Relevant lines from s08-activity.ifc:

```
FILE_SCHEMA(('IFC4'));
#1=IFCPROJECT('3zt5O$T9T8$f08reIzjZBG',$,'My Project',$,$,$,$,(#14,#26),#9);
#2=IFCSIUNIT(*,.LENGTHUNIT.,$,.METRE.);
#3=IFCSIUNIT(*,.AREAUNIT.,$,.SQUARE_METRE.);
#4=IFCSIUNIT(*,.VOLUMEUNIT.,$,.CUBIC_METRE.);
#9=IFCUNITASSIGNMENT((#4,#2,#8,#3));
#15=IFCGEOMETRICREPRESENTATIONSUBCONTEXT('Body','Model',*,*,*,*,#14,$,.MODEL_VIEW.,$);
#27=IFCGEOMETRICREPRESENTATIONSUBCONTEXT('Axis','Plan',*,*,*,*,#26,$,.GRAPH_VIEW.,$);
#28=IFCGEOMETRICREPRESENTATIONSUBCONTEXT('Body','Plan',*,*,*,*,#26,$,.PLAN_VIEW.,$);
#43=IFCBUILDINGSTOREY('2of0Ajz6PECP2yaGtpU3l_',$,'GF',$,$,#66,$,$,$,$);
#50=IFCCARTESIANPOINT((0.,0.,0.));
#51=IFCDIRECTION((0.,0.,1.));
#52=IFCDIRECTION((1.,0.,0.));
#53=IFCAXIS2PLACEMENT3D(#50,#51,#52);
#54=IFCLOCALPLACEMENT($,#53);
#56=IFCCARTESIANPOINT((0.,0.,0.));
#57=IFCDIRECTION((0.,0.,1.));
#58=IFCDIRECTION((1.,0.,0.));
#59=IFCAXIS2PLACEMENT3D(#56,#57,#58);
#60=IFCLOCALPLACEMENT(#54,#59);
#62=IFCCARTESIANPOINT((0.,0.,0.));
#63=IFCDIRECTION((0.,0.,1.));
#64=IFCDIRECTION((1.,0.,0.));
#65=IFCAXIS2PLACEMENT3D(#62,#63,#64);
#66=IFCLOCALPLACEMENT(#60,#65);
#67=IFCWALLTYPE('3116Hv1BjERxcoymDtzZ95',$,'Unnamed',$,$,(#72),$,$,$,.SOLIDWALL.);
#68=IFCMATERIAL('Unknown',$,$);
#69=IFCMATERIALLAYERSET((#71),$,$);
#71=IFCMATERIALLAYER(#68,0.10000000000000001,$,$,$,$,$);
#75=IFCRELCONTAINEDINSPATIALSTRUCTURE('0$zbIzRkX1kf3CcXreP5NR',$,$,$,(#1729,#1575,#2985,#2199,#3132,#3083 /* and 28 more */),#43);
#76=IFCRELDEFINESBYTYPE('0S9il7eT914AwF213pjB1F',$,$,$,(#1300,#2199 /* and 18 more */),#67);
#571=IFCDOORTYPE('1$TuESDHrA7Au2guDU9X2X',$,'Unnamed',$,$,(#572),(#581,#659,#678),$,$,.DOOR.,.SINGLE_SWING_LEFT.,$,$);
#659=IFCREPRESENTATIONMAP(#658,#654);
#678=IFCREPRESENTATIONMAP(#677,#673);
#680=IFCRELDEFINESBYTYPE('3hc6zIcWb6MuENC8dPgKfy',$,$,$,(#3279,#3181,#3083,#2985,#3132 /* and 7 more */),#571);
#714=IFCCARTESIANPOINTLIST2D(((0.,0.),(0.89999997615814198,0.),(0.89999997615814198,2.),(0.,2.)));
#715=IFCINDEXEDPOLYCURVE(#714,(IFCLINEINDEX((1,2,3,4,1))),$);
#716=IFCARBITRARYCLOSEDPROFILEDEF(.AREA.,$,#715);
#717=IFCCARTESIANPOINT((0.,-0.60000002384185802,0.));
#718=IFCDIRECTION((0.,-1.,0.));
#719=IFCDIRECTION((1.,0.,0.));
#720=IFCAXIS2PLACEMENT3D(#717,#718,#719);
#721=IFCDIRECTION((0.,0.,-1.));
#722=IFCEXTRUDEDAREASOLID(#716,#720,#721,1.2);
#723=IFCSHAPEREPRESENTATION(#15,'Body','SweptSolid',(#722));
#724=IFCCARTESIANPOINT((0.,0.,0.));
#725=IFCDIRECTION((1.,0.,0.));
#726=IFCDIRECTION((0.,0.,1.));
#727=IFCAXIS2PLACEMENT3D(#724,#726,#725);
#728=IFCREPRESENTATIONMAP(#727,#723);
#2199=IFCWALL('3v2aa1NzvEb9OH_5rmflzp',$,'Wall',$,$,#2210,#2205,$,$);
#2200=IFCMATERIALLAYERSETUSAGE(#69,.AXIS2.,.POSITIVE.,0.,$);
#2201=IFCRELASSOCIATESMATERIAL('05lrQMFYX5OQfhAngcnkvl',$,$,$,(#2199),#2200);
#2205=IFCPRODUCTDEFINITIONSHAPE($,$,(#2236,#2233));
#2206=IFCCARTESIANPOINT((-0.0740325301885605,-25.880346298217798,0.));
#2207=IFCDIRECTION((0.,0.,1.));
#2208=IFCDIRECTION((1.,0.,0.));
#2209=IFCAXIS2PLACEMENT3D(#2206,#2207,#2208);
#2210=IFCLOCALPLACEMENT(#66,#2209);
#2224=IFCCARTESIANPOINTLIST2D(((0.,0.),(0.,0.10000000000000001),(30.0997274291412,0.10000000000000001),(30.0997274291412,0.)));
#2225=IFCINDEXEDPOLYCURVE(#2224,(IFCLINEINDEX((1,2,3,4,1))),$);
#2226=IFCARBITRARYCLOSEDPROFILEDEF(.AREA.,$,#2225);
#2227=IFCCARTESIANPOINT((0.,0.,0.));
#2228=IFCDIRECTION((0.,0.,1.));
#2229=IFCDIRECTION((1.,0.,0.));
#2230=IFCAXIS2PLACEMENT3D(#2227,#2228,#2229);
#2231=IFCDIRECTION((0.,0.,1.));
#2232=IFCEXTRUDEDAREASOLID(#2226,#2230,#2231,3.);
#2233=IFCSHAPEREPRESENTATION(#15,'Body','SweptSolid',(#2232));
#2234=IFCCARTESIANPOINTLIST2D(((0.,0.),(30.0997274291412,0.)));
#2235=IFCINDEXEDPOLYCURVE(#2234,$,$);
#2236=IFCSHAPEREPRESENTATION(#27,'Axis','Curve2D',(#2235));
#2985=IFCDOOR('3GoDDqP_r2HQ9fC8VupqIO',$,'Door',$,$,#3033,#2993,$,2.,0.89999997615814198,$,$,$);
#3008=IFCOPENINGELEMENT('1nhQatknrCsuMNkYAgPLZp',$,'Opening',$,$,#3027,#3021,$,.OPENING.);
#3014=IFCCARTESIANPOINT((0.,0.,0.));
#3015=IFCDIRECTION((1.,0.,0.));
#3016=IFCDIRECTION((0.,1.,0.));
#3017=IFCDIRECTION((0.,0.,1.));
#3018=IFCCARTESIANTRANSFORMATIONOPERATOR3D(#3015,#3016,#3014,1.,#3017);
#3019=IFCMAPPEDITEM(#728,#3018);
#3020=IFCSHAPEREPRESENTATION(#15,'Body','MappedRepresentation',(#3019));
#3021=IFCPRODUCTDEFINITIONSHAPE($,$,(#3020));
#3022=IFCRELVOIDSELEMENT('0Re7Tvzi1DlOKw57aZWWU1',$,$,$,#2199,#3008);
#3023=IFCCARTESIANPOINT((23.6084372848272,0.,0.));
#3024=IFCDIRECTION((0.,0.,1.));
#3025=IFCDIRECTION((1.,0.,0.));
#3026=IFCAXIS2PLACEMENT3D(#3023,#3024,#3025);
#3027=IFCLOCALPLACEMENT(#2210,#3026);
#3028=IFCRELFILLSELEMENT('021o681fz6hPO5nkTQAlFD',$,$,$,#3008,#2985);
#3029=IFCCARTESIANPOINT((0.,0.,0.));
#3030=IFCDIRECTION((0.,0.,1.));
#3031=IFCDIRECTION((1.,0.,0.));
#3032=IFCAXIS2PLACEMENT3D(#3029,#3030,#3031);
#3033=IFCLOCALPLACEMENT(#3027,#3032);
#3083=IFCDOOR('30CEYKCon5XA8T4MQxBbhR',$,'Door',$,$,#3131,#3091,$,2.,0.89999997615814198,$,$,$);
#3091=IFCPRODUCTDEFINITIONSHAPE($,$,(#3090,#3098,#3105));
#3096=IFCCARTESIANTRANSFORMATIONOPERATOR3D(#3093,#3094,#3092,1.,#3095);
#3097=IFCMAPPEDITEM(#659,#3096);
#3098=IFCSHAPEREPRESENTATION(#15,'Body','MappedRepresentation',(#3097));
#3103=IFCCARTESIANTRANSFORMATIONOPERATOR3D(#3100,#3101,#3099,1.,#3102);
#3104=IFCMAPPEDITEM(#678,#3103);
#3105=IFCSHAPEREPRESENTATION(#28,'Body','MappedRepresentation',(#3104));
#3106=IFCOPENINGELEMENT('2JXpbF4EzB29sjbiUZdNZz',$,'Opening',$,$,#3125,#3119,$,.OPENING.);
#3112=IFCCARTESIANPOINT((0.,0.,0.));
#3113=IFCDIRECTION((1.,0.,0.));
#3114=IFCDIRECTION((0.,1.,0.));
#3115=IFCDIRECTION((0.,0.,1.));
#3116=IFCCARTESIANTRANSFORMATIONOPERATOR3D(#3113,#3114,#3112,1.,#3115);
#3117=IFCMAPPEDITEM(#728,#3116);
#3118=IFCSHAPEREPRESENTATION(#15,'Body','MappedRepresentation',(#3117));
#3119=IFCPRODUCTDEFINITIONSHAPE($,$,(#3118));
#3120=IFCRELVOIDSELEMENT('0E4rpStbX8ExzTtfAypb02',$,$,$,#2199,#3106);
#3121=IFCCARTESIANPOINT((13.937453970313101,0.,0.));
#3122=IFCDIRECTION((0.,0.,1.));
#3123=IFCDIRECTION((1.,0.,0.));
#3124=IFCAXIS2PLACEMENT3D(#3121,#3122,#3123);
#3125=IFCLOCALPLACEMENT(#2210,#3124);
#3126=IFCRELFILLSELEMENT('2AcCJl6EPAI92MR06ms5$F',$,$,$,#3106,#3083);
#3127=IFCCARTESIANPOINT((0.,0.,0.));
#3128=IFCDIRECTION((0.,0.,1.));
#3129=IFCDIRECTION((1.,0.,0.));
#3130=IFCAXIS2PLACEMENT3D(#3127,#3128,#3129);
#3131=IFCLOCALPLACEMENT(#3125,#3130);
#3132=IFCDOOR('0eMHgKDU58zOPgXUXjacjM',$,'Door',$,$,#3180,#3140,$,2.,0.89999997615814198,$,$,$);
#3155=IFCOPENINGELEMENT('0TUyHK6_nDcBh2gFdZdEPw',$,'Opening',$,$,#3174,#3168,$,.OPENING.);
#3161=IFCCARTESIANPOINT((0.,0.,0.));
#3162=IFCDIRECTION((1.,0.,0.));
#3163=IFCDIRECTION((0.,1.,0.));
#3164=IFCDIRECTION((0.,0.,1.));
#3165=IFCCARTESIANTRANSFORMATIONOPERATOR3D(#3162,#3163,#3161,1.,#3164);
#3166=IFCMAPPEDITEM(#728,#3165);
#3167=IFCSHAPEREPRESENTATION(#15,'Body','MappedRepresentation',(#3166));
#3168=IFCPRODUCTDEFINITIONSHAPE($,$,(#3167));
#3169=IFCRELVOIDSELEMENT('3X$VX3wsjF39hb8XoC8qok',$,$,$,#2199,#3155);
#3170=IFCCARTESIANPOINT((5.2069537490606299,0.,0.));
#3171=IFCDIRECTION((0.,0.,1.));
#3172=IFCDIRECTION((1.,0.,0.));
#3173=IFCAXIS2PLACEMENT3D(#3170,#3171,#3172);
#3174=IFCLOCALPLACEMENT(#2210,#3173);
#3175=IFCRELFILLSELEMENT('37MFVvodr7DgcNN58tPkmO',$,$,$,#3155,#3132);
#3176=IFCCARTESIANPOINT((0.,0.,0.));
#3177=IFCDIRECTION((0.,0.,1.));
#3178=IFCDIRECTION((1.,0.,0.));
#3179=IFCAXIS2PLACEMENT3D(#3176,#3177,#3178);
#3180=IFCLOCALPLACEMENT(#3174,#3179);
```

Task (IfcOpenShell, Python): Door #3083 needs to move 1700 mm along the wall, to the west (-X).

```python
import ifcopenshell
import ifcopenshell.api.geometry
import ifcopenshell.util.placement
import ifcopenshell.util.unit

model = ifcopenshell.open("s08-activity.ifc")
unit_scale = ifcopenshell.util.unit.calculate_unit_scale(model)

door = model.by_guid("30CEYKCon5XA8T4MQxBbhR")
opening = door.FillsVoids[0].RelatingOpeningElement
wall = opening.VoidsElements[0].RelatingBuildingElement

wall_matrix = ifcopenshell.util.placement.get_local_placement(wall.ObjectPlacement)
shift = wall_matrix[:3, 0] * -1.7 / unit_scale
before = ifcopenshell.util.placement.get_local_placement(door.ObjectPlacement)[:3, 3].copy()

# The door is placed relative to its opening, so it follows when the opening moves.
matrix = ifcopenshell.util.placement.get_local_placement(opening.ObjectPlacement)
matrix[:3, 3] += shift
ifcopenshell.api.geometry.edit_object_placement(
    model, product=opening, matrix=matrix, is_si=False, should_transform_children=True
)

after = ifcopenshell.util.placement.get_local_placement(door.ObjectPlacement)[:3, 3]
print("door moved by", (after - before).round(3) + 0.0)

model.write("s08-activity_rev.ifc")
```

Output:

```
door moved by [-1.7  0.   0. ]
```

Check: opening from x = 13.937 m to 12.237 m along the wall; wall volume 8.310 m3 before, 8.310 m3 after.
